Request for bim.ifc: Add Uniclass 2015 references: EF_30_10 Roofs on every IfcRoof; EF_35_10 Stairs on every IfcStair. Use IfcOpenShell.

First a look at what the model holds.

```python
import ifcopenshell

model = ifcopenshell.open("bim.ifc")
print(model.schema)
print("classifications:", [c.Name for c in model.by_type("IfcClassification")])
for ifc_class in ("IfcDoor", "IfcRoof", "IfcStair", "IfcWall", "IfcWindow"):
    print(ifc_class, len(model.by_type(ifc_class)))
```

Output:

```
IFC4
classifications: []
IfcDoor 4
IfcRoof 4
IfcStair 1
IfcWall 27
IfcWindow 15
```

```python
import ifcopenshell
import ifcopenshell.api.classification

model = ifcopenshell.open("bim.ifc")

system = ifcopenshell.api.classification.add_classification(model, classification="Uniclass 2015")

codes = {
    "IfcRoof": ("EF_30_10", "Roofs"),
    "IfcStair": ("EF_35_10", "Stairs"),
}
for ifc_class, (code, name) in codes.items():
    products = model.by_type(ifc_class)
    ifcopenshell.api.classification.add_reference(
        model, products=products, classification=system, identification=code, name=name
    )
    print(code, len(products))

model.write("bim_updated.ifc")
```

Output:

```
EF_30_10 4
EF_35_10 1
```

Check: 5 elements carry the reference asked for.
